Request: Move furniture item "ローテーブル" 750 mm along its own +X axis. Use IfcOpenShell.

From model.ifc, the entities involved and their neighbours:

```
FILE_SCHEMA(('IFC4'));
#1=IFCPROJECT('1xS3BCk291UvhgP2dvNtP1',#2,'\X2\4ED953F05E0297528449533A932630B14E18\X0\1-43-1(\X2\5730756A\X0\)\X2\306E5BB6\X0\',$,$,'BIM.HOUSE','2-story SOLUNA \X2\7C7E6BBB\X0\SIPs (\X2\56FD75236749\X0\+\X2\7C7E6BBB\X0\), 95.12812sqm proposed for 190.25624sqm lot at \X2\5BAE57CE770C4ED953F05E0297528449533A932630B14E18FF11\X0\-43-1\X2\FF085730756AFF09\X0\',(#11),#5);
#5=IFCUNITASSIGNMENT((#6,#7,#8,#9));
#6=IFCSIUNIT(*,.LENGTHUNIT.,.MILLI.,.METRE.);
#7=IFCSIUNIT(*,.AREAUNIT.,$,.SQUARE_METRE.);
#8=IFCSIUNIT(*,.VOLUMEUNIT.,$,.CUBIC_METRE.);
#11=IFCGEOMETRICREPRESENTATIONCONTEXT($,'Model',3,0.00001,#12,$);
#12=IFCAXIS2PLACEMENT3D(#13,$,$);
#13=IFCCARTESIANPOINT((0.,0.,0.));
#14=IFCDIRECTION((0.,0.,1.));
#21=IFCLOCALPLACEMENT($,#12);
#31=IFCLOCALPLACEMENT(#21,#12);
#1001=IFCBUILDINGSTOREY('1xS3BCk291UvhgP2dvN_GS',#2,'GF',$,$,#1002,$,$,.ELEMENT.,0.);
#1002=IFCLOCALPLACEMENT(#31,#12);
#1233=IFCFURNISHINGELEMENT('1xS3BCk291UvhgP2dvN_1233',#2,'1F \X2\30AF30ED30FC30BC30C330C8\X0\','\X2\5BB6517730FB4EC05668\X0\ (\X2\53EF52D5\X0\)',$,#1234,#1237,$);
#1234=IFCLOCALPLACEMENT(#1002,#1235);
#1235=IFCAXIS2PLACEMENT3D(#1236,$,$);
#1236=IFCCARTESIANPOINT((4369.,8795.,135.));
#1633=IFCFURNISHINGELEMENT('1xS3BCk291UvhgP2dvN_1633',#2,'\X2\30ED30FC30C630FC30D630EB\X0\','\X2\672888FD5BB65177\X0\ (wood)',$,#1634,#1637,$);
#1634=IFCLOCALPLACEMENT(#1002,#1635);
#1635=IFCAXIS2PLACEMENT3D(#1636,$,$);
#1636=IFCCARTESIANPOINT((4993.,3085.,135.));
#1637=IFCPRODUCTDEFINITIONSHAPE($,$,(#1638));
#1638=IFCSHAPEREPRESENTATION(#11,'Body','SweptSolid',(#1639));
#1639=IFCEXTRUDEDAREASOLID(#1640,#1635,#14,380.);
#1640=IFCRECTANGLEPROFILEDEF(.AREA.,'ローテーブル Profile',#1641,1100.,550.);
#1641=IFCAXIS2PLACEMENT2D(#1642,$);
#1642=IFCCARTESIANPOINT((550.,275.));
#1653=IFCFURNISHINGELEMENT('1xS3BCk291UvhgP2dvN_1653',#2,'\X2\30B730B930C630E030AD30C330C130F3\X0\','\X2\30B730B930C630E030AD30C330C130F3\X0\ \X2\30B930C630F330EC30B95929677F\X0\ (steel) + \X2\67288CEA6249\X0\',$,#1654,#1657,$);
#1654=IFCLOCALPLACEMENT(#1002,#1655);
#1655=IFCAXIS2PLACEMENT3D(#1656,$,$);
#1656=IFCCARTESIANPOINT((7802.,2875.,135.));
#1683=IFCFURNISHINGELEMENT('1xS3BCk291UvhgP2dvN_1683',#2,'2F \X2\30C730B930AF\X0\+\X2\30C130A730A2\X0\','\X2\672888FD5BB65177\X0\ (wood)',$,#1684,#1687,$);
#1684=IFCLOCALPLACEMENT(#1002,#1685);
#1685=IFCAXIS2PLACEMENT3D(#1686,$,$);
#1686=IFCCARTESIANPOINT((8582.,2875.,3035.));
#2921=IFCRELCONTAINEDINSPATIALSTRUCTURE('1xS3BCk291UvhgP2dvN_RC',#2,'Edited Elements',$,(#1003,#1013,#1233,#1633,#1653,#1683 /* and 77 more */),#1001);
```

```python
import ifcopenshell
import ifcopenshell.api.geometry
import ifcopenshell.util.placement
import ifcopenshell.util.unit

model = ifcopenshell.open("model.ifc")
unit_scale = ifcopenshell.util.unit.calculate_unit_scale(model)

item = model.by_guid("1xS3BCk291UvhgP2dvN_1633")
matrix = ifcopenshell.util.placement.get_local_placement(item.ObjectPlacement)
matrix[:3, 3] += matrix[:3, 0] * 0.75 / unit_scale
ifcopenshell.api.geometry.edit_object_placement(model, product=item, matrix=matrix, is_si=False)

print(ifcopenshell.util.placement.get_local_placement(item.ObjectPlacement).round(3) + 0.0)

model.write("model-out.ifc")
```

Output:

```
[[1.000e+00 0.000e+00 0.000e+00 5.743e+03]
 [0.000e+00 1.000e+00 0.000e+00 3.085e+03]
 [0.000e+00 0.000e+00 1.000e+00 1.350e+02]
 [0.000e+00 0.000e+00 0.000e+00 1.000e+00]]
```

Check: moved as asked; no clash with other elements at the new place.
